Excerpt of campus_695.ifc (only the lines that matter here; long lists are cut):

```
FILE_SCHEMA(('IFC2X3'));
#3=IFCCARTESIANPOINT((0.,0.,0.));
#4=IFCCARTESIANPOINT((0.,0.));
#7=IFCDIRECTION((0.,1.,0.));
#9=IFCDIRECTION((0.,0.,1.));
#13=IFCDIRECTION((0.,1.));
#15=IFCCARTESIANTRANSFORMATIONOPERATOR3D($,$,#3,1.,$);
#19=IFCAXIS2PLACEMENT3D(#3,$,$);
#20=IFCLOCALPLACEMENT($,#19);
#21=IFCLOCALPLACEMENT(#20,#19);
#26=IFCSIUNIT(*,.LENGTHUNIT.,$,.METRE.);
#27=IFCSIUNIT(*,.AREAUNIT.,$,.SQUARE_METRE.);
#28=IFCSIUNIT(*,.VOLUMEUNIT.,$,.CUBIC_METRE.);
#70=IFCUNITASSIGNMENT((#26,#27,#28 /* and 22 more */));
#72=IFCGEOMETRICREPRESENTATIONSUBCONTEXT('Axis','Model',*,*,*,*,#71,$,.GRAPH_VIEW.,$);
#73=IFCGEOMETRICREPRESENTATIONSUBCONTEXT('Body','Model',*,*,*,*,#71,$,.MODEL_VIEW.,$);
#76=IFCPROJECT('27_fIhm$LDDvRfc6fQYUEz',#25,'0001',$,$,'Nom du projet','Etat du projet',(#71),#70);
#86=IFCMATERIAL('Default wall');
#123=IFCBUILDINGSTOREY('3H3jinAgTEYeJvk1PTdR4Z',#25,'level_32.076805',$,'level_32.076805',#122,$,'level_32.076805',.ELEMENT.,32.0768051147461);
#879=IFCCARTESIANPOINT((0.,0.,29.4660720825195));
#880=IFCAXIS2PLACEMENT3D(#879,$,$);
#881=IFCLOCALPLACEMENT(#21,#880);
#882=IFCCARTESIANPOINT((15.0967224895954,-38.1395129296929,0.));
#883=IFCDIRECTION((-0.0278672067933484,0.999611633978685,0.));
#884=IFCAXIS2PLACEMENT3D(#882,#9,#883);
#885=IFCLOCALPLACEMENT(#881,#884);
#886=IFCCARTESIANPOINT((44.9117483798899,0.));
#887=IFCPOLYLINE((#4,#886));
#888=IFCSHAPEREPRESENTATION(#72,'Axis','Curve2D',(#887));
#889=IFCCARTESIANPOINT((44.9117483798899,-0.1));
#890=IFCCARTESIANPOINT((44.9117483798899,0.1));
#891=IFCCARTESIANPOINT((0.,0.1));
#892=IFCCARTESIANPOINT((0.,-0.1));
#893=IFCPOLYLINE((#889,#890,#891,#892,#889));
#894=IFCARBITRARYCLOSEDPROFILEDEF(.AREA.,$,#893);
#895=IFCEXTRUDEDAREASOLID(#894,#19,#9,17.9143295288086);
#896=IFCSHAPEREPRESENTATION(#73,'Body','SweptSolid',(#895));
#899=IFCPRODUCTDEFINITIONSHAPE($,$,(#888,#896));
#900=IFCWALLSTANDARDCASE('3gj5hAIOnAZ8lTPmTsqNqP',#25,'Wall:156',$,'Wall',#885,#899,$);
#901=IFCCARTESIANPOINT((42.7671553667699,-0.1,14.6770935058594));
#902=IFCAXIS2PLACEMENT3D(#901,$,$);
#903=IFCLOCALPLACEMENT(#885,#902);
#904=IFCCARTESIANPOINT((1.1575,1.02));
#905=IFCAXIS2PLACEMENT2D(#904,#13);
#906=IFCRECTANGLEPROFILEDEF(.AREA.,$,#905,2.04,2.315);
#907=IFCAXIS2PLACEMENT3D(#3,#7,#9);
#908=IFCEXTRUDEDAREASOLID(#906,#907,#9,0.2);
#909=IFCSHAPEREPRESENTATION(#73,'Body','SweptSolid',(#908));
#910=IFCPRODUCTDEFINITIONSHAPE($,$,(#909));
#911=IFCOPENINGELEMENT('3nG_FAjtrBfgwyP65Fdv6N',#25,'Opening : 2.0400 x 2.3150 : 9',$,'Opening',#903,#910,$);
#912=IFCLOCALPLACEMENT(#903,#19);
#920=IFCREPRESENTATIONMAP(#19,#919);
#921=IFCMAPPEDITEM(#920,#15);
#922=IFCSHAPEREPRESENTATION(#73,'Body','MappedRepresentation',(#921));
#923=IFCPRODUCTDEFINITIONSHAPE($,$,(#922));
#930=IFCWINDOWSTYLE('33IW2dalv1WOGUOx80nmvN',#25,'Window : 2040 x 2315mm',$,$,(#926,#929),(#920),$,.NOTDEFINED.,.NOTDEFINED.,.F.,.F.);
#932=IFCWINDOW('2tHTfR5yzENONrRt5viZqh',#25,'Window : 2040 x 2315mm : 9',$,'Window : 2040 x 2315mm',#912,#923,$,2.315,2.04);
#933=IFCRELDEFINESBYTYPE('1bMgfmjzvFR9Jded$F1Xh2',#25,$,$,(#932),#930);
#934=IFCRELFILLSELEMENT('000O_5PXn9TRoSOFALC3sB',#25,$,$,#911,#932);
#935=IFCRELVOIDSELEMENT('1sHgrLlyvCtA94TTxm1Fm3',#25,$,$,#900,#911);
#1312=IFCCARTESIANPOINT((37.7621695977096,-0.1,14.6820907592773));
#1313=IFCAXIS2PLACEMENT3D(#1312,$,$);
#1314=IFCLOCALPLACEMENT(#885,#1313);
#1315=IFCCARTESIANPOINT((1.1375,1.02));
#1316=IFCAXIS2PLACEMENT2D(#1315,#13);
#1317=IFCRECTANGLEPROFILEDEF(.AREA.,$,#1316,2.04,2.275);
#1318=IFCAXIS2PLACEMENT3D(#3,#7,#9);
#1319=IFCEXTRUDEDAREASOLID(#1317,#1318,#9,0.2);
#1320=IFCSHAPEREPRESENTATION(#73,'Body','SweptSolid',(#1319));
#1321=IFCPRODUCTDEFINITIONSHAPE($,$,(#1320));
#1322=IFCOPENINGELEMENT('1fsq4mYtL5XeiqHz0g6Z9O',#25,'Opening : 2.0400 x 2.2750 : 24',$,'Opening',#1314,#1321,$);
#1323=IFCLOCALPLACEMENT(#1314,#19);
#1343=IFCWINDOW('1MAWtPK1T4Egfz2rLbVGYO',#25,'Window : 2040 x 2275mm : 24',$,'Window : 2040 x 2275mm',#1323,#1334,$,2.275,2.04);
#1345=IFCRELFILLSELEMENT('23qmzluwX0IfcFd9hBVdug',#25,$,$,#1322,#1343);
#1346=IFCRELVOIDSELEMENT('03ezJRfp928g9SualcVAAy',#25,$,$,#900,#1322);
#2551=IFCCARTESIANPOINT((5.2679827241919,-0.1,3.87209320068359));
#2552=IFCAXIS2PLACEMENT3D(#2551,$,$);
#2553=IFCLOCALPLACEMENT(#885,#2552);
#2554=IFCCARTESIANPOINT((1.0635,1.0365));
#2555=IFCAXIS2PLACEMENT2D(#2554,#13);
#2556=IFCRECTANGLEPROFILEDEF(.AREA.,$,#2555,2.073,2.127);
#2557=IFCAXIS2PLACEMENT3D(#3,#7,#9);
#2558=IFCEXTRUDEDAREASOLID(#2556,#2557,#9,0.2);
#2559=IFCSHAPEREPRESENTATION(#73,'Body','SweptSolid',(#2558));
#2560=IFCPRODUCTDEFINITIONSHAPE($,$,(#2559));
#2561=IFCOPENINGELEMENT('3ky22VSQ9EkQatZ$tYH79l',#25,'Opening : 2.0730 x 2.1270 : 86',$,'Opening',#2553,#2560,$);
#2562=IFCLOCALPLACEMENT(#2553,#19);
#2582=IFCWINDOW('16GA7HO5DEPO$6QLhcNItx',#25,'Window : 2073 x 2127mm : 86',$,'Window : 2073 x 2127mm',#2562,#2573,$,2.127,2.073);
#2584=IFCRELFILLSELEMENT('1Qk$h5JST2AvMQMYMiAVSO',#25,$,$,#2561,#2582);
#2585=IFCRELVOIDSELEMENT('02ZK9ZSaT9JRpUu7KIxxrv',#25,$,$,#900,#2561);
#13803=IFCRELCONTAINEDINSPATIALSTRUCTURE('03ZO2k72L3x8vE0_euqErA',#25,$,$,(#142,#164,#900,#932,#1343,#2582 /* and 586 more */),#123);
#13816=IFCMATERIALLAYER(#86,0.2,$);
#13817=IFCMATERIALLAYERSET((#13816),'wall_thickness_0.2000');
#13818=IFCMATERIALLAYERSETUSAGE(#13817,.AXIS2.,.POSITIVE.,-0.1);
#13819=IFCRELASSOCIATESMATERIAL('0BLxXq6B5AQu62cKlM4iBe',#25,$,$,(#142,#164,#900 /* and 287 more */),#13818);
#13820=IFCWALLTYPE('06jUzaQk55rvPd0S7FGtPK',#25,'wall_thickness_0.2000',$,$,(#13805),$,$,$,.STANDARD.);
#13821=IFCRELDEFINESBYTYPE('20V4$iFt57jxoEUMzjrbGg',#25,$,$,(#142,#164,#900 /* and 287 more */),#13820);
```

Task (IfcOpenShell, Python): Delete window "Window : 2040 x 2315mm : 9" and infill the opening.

```python
import ifcopenshell
import ifcopenshell.api.feature
import ifcopenshell.api.root
import ifcopenshell.geom
import ifcopenshell.util.shape

model = ifcopenshell.open("campus_695.ifc")
settings = ifcopenshell.geom.settings()


def volume(element):
    """Net volume in cubic metres, openings subtracted."""
    shape = ifcopenshell.geom.create_shape(settings, element)
    return ifcopenshell.util.shape.get_volume(shape.geometry)


window = model.by_guid("2tHTfR5yzENONrRt5viZqh")
opening = window.FillsVoids[0].RelatingOpeningElement
wall = opening.VoidsElements[0].RelatingBuildingElement
before = volume(wall)

ifcopenshell.api.root.remove_product(model, product=window)
ifcopenshell.api.feature.remove_feature(model, feature=opening)

after = volume(wall)

print(f"wall volume {before:.3f} -> {after:.3f} m3")

model.write("campus_695_v2.ifc")
```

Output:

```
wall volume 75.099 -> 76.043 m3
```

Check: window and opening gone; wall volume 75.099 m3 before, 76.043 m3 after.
